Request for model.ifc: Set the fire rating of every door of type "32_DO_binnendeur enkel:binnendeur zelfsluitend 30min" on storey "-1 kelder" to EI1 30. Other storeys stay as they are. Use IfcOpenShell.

First a look at what the model holds.

```python
import ifcopenshell
import ifcopenshell.util.element

model = ifcopenshell.open("model.ifc")
print(model.schema)
storey = next(s for s in model.by_type("IfcBuildingStorey") if s.Name == "-1 kelder")
doors = [e for e in ifcopenshell.util.element.get_decomposition(storey) if e.is_a("IfcDoor")]
seen = {}
for e in doors:
    element_type = ifcopenshell.util.element.get_type(e)
    key = (element_type.Name if element_type != e and element_type else None, ifcopenshell.util.element.get_pset(e, "Pset_DoorCommon", "FireRating"))
    seen[key] = seen.get(key, 0) + 1
for (name, value), count in sorted(seen.items(), key=str):
    print(count, "x", name, "|", value)
```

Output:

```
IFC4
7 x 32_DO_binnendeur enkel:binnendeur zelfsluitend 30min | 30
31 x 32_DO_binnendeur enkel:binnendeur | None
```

```python
import ifcopenshell
import ifcopenshell.api.pset
import ifcopenshell.util.element

model = ifcopenshell.open("model.ifc")

storey = next(s for s in model.by_type("IfcBuildingStorey") if s.Name == "-1 kelder")
doors = [e for e in ifcopenshell.util.element.get_decomposition(storey) if e.is_a("IfcDoor")]

count = 0
for e in doors:
    element_type = ifcopenshell.util.element.get_type(e)
    if element_type in (None, e) or element_type.Name != "32_DO_binnendeur enkel:binnendeur zelfsluitend 30min":
        continue
    # add_pset returns the element's existing set when there is one.
    pset = ifcopenshell.api.pset.add_pset(model, product=e, name="Pset_DoorCommon")
    ifcopenshell.api.pset.edit_pset(model, pset=pset, properties={"FireRating": "EI1 30"})
    count += 1

print(count, "doors updated")

model.write("model-out.ifc")
```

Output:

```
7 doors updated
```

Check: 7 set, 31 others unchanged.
